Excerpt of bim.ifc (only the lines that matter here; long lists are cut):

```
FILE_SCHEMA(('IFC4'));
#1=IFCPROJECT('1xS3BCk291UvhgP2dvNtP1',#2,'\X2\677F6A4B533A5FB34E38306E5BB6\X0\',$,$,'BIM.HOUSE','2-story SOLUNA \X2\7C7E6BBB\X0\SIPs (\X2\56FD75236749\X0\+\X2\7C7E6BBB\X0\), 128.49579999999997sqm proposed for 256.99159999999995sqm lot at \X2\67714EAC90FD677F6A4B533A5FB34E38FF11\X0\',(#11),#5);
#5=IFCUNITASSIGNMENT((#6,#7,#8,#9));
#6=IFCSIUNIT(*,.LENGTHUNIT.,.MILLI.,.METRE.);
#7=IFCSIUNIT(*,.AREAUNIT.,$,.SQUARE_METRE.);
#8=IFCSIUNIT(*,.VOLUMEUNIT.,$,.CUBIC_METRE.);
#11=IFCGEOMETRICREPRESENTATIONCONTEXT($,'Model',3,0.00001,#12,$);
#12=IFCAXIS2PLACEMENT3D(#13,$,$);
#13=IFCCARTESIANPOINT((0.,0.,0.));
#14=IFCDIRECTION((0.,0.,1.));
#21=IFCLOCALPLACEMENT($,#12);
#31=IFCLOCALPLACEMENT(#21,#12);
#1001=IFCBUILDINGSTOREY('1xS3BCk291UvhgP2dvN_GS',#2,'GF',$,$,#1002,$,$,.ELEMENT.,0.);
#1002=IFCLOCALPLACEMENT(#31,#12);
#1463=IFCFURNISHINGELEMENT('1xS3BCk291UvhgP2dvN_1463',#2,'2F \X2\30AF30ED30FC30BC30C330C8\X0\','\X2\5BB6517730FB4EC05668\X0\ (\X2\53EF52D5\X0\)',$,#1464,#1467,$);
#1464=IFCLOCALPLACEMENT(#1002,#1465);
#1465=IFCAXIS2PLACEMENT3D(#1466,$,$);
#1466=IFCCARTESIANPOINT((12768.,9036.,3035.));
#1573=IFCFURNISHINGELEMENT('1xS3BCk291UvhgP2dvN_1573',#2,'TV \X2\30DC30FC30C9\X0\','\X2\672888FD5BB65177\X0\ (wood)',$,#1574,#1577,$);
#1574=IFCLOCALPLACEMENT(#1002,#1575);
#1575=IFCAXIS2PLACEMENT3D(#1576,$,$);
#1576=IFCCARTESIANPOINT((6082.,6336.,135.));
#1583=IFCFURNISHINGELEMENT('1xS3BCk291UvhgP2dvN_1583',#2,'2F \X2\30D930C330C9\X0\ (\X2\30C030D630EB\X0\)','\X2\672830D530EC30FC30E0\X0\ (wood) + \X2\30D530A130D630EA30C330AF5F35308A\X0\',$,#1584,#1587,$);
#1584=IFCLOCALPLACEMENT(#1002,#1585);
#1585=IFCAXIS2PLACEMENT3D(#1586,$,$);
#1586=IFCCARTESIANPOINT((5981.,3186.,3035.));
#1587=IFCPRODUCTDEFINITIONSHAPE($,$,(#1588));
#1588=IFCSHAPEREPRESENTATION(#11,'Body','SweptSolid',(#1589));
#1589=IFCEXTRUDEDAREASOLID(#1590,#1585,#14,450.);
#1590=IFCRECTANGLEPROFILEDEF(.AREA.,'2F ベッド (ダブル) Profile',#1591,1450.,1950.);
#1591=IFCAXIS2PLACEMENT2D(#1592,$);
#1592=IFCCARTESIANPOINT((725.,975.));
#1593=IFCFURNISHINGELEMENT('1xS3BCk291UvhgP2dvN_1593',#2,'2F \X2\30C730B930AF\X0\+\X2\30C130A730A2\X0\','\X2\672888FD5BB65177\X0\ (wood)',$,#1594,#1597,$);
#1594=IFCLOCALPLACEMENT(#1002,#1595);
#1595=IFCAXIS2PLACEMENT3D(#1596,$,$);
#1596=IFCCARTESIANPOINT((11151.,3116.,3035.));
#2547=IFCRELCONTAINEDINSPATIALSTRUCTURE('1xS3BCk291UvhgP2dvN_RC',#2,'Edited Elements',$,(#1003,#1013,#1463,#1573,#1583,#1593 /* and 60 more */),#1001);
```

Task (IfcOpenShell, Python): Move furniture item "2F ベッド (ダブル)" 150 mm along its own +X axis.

```python
import ifcopenshell
import ifcopenshell.api.geometry
import ifcopenshell.util.placement
import ifcopenshell.util.unit

model = ifcopenshell.open("bim.ifc")
unit_scale = ifcopenshell.util.unit.calculate_unit_scale(model)

item = model.by_guid("1xS3BCk291UvhgP2dvN_1583")
matrix = ifcopenshell.util.placement.get_local_placement(item.ObjectPlacement)
matrix[:3, 3] += matrix[:3, 0] * 0.15 / unit_scale
ifcopenshell.api.geometry.edit_object_placement(model, product=item, matrix=matrix, is_si=False)

print(ifcopenshell.util.placement.get_local_placement(item.ObjectPlacement).round(3) + 0.0)

model.write("bim_edited.ifc")
```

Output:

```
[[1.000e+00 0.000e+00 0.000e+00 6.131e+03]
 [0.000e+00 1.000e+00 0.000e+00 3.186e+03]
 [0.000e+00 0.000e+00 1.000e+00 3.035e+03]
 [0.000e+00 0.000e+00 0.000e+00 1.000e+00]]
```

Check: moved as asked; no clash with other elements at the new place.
